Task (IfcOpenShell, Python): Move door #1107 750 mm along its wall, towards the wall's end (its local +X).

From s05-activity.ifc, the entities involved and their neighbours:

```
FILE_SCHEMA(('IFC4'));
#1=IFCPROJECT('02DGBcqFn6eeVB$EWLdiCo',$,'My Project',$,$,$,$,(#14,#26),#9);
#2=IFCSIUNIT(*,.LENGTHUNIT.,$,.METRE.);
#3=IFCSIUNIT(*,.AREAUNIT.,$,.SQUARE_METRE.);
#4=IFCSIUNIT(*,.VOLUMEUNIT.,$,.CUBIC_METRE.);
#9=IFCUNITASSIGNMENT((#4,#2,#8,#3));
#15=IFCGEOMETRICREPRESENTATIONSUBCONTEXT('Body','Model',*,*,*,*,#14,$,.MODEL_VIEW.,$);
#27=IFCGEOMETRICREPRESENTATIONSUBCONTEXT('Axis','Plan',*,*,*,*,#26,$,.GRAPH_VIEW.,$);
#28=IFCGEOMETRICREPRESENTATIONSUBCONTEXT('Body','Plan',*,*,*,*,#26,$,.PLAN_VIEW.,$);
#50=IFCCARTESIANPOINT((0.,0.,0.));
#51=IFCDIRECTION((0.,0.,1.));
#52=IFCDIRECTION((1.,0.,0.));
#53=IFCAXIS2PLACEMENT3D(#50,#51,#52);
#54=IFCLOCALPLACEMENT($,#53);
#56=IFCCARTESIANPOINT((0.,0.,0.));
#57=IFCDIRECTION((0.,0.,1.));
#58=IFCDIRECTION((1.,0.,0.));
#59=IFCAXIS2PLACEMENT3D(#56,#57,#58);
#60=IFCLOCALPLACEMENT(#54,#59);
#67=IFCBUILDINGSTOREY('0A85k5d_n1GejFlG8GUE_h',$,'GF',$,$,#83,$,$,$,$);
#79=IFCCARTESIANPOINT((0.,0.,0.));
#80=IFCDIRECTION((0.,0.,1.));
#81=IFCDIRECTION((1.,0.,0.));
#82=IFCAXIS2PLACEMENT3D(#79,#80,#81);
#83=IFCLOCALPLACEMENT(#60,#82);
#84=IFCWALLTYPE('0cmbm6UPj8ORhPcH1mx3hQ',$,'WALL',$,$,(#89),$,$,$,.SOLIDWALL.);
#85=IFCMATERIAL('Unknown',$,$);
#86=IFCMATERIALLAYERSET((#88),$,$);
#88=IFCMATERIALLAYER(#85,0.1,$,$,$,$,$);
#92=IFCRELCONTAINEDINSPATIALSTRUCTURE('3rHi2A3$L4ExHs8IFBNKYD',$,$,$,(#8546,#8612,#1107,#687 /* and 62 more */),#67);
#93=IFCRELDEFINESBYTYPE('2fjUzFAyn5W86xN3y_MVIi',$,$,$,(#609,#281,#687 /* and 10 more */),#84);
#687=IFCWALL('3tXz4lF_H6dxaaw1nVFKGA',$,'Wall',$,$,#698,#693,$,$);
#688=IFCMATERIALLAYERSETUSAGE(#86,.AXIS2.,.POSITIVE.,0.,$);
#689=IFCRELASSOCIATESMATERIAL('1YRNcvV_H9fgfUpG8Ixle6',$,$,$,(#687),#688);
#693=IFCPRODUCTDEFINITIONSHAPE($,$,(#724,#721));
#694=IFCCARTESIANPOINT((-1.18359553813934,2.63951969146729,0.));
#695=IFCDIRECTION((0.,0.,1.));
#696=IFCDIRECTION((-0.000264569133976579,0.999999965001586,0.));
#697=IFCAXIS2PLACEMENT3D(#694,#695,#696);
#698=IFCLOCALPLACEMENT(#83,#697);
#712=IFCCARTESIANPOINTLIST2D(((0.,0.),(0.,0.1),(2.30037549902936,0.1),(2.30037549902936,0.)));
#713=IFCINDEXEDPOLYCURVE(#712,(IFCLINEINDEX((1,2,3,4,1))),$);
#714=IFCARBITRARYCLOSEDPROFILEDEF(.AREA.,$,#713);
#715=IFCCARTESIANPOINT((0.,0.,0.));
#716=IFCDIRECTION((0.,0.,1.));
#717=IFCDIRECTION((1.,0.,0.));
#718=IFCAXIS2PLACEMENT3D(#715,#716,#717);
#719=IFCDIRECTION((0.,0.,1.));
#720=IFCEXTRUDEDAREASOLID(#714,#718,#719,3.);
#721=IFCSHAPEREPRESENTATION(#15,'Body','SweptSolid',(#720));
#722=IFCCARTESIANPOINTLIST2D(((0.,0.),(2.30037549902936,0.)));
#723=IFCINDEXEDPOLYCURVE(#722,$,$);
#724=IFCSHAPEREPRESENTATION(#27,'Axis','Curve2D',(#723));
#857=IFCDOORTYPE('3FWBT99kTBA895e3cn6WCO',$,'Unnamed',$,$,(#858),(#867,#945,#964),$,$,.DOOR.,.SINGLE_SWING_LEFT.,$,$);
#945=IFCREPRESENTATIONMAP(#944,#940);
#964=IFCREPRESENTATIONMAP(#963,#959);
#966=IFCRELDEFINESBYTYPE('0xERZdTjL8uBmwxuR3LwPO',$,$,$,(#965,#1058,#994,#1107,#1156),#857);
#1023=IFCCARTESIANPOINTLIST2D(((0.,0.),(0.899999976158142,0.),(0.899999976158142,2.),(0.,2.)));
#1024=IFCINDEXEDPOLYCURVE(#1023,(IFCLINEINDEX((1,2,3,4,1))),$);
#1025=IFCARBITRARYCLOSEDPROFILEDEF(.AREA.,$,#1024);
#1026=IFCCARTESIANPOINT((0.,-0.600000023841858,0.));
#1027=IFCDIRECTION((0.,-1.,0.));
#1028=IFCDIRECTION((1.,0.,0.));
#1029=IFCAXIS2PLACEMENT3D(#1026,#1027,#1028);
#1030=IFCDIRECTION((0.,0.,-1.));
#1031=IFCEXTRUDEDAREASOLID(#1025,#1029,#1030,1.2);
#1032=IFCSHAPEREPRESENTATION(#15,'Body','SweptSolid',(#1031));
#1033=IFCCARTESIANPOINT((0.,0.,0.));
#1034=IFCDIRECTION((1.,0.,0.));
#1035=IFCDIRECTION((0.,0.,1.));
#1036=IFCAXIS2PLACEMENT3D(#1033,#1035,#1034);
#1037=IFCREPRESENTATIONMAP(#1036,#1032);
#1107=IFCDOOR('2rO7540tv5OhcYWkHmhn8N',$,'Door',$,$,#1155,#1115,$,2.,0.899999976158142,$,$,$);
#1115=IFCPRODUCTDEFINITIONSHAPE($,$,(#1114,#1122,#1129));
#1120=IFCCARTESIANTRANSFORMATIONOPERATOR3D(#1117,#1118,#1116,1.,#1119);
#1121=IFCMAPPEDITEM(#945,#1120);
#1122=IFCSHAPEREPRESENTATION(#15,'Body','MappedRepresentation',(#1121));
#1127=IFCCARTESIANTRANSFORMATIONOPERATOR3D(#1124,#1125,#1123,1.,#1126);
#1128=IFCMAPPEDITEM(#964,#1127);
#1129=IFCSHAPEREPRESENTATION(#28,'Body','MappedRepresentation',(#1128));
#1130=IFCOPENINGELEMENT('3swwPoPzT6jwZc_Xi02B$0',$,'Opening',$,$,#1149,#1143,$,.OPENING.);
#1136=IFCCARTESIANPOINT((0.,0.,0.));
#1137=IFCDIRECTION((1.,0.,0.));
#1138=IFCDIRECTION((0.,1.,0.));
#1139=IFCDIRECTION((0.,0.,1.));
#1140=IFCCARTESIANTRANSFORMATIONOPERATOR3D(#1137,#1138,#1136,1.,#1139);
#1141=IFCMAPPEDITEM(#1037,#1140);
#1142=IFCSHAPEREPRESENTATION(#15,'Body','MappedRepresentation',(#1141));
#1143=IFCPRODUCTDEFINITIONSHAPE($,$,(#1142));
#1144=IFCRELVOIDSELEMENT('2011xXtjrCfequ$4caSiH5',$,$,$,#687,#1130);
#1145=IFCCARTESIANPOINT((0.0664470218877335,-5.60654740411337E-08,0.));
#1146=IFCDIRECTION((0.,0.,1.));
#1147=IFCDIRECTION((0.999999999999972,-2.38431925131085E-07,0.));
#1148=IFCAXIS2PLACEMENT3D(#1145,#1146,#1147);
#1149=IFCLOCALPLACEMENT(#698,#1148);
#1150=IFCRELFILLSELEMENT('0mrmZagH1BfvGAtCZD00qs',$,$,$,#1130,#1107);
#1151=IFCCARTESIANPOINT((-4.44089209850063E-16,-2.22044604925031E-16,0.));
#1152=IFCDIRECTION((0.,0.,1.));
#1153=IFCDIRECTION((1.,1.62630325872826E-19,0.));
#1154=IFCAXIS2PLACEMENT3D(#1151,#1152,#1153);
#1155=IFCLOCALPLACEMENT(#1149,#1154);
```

```python
import ifcopenshell
import ifcopenshell.api.geometry
import ifcopenshell.util.placement

model = ifcopenshell.open("s05-activity.ifc")

door = model.by_guid("2rO7540tv5OhcYWkHmhn8N")
opening = door.FillsVoids[0].RelatingOpeningElement
wall = opening.VoidsElements[0].RelatingBuildingElement

wall_matrix = ifcopenshell.util.placement.get_local_placement(wall.ObjectPlacement)
shift = wall_matrix[:3, 0] * 0.75
before = ifcopenshell.util.placement.get_local_placement(door.ObjectPlacement)[:3, 3].copy()

# The door is placed relative to its opening, so it follows when the opening moves.
matrix = ifcopenshell.util.placement.get_local_placement(opening.ObjectPlacement)
matrix[:3, 3] += shift
ifcopenshell.api.geometry.edit_object_placement(
    model, product=opening, matrix=matrix, is_si=False, should_transform_children=True
)

after = ifcopenshell.util.placement.get_local_placement(door.ObjectPlacement)[:3, 3]
print("door moved by", (after - before).round(3) + 0.0)

model.write("s05-activity-out.ifc")
```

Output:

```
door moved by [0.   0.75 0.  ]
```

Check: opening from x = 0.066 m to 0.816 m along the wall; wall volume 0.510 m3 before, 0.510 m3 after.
